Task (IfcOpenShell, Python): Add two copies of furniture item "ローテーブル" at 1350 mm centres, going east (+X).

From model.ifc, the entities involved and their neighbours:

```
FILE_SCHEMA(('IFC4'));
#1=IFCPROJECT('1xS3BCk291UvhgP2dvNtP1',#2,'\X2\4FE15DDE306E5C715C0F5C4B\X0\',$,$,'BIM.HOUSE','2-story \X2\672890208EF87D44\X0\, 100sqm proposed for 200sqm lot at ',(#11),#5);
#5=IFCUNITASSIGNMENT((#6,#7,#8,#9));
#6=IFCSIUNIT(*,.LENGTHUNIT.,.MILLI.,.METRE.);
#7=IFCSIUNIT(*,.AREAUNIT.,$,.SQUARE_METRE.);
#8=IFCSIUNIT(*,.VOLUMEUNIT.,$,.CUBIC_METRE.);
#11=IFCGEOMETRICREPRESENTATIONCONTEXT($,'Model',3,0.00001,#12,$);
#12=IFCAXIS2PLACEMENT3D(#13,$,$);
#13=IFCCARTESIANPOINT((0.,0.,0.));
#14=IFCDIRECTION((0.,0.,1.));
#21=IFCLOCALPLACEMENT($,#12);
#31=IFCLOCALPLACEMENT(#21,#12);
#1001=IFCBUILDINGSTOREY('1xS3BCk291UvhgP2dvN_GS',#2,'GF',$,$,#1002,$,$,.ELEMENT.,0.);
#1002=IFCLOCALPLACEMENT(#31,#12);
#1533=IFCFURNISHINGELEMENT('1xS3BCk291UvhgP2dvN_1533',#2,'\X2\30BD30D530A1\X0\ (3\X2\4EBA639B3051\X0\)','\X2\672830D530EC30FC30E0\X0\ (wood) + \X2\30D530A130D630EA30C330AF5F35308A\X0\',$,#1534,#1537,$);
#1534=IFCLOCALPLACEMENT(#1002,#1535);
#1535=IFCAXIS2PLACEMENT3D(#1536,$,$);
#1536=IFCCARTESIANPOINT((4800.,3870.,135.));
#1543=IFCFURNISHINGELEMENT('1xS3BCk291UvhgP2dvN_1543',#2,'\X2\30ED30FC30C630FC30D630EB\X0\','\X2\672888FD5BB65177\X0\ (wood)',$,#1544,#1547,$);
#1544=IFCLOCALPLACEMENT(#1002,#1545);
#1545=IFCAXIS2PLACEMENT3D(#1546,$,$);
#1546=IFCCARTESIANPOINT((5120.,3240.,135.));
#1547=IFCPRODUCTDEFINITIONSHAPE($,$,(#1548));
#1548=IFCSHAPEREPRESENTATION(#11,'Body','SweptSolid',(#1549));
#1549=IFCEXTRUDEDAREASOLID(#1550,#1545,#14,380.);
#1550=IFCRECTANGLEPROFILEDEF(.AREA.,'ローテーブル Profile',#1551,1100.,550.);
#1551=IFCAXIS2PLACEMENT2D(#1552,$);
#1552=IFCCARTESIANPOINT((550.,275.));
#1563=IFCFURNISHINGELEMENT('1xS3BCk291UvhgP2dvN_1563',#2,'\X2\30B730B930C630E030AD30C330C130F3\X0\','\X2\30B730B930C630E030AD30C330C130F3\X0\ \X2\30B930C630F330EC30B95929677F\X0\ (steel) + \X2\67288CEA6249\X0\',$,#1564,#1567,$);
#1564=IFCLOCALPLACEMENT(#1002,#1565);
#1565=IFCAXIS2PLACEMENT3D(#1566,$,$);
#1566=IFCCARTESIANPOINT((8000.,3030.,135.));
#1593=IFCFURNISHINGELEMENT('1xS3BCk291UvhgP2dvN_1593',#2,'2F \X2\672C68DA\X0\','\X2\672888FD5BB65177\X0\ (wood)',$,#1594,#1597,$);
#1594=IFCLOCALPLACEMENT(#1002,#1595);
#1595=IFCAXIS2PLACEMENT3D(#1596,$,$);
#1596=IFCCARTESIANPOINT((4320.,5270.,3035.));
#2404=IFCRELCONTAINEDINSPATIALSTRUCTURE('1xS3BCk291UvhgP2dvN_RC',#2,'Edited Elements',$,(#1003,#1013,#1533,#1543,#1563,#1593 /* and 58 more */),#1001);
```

```python
import numpy as np
import ifcopenshell
import ifcopenshell.api.geometry
import ifcopenshell.api.root
import ifcopenshell.util.element
import ifcopenshell.util.placement
import ifcopenshell.util.unit

model = ifcopenshell.open("model.ifc")
unit_scale = ifcopenshell.util.unit.calculate_unit_scale(model)


def reuse_history(source, copy):
    """copy_class also copies each property set's owner history, people and application; keep the originals."""
    for rel in copy.IsDefinedBy:
        if rel.is_a("IfcRelDefinesByProperties") and (history := rel.RelatingPropertyDefinition.OwnerHistory):
            rel.RelatingPropertyDefinition.OwnerHistory = source.OwnerHistory
            ifcopenshell.util.element.remove_deep2(model, history)


source = model.by_guid("1xS3BCk291UvhgP2dvN_1543")
base = ifcopenshell.util.placement.get_local_placement(source.ObjectPlacement)
step = np.array([1.0, 0.0, 0.0]) * 1.35 / unit_scale

for i in range(1, 3):
    copy = ifcopenshell.api.root.copy_class(model, product=source)
    copy.Representation = ifcopenshell.util.element.copy_deep(
        model, source.Representation, exclude=["IfcGeometricRepresentationContext", "IfcRepresentationMap"]
    )
    reuse_history(source, copy)
    matrix = base.copy()
    matrix[:3, 3] += i * step
    print("added at", matrix[:3, 3].round(3) + 0.0)
    ifcopenshell.api.geometry.edit_object_placement(model, product=copy, matrix=matrix, is_si=False)

model.write("model-out.ifc")
```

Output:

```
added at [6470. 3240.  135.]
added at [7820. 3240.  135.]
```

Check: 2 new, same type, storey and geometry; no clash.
